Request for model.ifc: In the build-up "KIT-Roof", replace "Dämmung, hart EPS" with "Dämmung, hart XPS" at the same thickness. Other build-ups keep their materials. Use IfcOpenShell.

First a look at what the model holds.

```python
import ifcopenshell
import ifcopenshell.util.element

model = ifcopenshell.open("model.ifc")
print(model.schema)
for layer_set in model.by_type("IfcMaterialLayerSet"):
    if layer_set.LayerSetName == "KIT-Roof":
        for layer in layer_set.MaterialLayers:
            print(layer.id(), layer.Material and layer.Material.Name, layer.LayerThickness, sep=" | ")
        print(len(ifcopenshell.util.element.get_elements_by_material(model, layer_set)), "elements and types use it")
print(sorted(m.Name for m in model.by_type("IfcMaterial") if m.Name)[:60])
```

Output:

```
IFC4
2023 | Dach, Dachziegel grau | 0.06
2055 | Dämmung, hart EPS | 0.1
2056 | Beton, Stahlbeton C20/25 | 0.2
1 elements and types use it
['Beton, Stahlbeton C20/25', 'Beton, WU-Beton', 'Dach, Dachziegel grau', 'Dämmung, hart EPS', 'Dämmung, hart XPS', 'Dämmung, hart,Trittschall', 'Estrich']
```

```python
import ifcopenshell
import ifcopenshell.api.material

model = ifcopenshell.open("model.ifc")

layer_set = next(s for s in model.by_type("IfcMaterialLayerSet") if s.LayerSetName == "KIT-Roof")
layer = next(l for l in layer_set.MaterialLayers if l.Material and l.Material.Name == "Dämmung, hart EPS")
material = next(m for m in model.by_type("IfcMaterial") if m.Name == "Dämmung, hart XPS")

# Point this one layer at the other material; renaming the old one would change it everywhere.
ifcopenshell.api.material.edit_layer(model, layer=layer, attributes={}, material=material)

print([l.Material.Name if l.Material else None for l in layer_set.MaterialLayers])

model.write("model_updated.ifc")
```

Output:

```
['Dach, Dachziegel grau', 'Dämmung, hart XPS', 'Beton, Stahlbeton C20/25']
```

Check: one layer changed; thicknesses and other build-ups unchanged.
